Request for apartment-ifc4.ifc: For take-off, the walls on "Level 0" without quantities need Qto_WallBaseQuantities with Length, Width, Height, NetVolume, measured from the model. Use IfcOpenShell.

First a look at what the model holds.

```python
import ifcopenshell
import ifcopenshell.util.element
import ifcopenshell.util.unit

model = ifcopenshell.open("apartment-ifc4.ifc")
print(model.schema)
for unit_type in ("LENGTHUNIT", "AREAUNIT", "VOLUMEUNIT"):
    print(unit_type, ifcopenshell.util.unit.calculate_unit_scale(model, unit_type))
storey = next(s for s in model.by_type("IfcBuildingStorey") if s.Name == "Level 0")
walls = [e for e in ifcopenshell.util.element.get_decomposition(storey) if e.is_a("IfcWall")]
for e in sorted(walls, key=lambda e: e.id()):
    print(e.id(), e.is_a(), e.Name, list(ifcopenshell.util.element.get_psets(e, qtos_only=True)), sep=" | ")
```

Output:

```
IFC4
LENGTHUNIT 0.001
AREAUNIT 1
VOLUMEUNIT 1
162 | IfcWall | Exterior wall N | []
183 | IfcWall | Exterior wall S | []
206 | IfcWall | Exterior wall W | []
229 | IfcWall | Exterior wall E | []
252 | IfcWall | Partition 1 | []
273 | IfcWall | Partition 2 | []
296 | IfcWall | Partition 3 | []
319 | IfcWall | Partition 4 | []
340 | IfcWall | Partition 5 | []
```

```python
import ifcopenshell
import ifcopenshell.api.pset
import ifcopenshell.geom
import ifcopenshell.util.element
import ifcopenshell.util.shape
import ifcopenshell.util.unit

model = ifcopenshell.open("apartment-ifc4.ifc")
unit_scale = ifcopenshell.util.unit.calculate_unit_scale(model)
volume_scale = ifcopenshell.util.unit.calculate_unit_scale(model, "VOLUMEUNIT")
settings = ifcopenshell.geom.settings()

storey = next(s for s in model.by_type("IfcBuildingStorey") if s.Name == "Level 0")
walls = [e for e in ifcopenshell.util.element.get_decomposition(storey) if e.is_a("IfcWall")]

for e in sorted(walls, key=lambda e: e.id()):
    if ifcopenshell.util.element.get_psets(e, qtos_only=True, should_inherit=False):
        continue
    # Geometry comes back in metres, in the element's own axes.
    shape = ifcopenshell.geom.create_shape(settings, e)
    values = {
        "Length": ifcopenshell.util.shape.get_x(shape.geometry) / unit_scale,
        "Width": ifcopenshell.util.shape.get_y(shape.geometry) / unit_scale,
        "Height": ifcopenshell.util.shape.get_z(shape.geometry) / unit_scale,
        "NetVolume": ifcopenshell.util.shape.get_volume(shape.geometry) / volume_scale,
    }
    qto = ifcopenshell.api.pset.add_qto(model, product=e, name="Qto_WallBaseQuantities")
    ifcopenshell.api.pset.edit_qto(model, qto=qto, properties=values)
    print(e.id(), {k: round(v, 3) for k, v in values.items()})

model.write("apartment-ifc4_edited.ifc")
```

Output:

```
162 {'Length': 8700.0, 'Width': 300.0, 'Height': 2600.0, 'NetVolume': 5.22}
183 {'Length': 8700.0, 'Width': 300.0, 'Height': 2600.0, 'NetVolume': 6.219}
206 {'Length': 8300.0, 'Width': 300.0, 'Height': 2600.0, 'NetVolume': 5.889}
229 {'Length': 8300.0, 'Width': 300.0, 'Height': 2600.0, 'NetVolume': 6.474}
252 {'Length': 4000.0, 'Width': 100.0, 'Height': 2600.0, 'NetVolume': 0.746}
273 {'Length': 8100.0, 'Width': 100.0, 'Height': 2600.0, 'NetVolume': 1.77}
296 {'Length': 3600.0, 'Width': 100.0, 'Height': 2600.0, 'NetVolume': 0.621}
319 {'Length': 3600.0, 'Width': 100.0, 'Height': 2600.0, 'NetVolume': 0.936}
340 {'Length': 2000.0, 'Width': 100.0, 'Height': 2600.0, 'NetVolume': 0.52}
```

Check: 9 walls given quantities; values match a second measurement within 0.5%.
